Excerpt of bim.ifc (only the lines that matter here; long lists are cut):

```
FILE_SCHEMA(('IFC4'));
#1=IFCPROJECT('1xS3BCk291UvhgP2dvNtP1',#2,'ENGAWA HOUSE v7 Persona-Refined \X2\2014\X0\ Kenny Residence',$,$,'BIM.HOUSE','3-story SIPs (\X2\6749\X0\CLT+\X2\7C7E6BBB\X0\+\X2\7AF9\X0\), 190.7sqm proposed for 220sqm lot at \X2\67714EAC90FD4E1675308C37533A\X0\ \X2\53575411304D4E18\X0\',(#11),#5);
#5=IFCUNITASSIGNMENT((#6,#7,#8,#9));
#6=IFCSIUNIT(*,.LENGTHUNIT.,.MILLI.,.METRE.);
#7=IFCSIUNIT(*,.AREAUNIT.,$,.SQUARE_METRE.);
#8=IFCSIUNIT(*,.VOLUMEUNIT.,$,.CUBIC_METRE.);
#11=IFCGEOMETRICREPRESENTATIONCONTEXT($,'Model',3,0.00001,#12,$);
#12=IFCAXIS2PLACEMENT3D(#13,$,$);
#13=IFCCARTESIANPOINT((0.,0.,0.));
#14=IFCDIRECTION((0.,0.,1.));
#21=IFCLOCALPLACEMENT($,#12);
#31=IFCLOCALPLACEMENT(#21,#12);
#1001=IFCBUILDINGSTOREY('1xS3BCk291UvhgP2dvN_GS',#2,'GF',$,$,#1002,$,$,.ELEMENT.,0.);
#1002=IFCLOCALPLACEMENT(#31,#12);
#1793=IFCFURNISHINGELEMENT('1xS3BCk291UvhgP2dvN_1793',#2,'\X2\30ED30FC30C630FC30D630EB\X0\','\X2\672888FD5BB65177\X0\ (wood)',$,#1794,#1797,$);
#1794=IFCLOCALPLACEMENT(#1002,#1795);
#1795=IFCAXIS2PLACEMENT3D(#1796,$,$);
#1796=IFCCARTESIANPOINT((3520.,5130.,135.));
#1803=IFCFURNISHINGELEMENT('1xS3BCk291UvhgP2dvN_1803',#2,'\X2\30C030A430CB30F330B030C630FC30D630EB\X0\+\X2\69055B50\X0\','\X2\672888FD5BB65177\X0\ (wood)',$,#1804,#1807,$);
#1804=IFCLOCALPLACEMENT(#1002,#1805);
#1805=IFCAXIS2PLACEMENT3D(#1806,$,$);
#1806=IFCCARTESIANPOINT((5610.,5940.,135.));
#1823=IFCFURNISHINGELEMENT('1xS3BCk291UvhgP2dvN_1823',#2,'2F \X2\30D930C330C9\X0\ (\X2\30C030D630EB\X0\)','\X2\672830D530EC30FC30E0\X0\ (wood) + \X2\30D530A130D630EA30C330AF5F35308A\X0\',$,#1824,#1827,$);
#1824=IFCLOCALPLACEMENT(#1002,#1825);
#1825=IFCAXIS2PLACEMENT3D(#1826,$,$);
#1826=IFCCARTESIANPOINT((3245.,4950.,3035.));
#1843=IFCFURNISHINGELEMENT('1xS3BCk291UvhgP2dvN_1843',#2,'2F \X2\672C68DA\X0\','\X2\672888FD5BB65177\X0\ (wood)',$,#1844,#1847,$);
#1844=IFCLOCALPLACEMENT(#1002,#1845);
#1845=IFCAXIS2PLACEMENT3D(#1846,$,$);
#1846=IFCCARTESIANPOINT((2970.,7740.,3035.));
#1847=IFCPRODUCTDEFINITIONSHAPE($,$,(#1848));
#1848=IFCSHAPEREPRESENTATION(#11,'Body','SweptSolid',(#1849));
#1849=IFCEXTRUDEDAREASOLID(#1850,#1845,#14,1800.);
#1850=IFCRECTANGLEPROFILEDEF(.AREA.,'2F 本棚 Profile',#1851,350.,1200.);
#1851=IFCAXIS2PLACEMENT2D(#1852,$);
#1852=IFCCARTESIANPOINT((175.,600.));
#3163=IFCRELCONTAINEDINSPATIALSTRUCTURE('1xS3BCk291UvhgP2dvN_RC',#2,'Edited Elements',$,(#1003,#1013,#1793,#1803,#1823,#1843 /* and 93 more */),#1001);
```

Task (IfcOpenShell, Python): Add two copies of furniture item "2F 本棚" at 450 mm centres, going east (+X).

```python
import numpy as np
import ifcopenshell
import ifcopenshell.api.geometry
import ifcopenshell.api.root
import ifcopenshell.util.element
import ifcopenshell.util.placement
import ifcopenshell.util.unit

model = ifcopenshell.open("bim.ifc")
unit_scale = ifcopenshell.util.unit.calculate_unit_scale(model)


def reuse_history(source, copy):
    """copy_class also copies each property set's owner history, people and application; keep the originals."""
    for rel in copy.IsDefinedBy:
        if rel.is_a("IfcRelDefinesByProperties") and (history := rel.RelatingPropertyDefinition.OwnerHistory):
            rel.RelatingPropertyDefinition.OwnerHistory = source.OwnerHistory
            ifcopenshell.util.element.remove_deep2(model, history)


source = model.by_guid("1xS3BCk291UvhgP2dvN_1843")
base = ifcopenshell.util.placement.get_local_placement(source.ObjectPlacement)
step = np.array([1.0, 0.0, 0.0]) * 0.45 / unit_scale

for i in range(1, 3):
    copy = ifcopenshell.api.root.copy_class(model, product=source)
    copy.Representation = ifcopenshell.util.element.copy_deep(
        model, source.Representation, exclude=["IfcGeometricRepresentationContext", "IfcRepresentationMap"]
    )
    reuse_history(source, copy)
    matrix = base.copy()
    matrix[:3, 3] += i * step
    print("added at", matrix[:3, 3].round(3) + 0.0)
    ifcopenshell.api.geometry.edit_object_placement(model, product=copy, matrix=matrix, is_si=False)

model.write("bim_rev.ifc")
```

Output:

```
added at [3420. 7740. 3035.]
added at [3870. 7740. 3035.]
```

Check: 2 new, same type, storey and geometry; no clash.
